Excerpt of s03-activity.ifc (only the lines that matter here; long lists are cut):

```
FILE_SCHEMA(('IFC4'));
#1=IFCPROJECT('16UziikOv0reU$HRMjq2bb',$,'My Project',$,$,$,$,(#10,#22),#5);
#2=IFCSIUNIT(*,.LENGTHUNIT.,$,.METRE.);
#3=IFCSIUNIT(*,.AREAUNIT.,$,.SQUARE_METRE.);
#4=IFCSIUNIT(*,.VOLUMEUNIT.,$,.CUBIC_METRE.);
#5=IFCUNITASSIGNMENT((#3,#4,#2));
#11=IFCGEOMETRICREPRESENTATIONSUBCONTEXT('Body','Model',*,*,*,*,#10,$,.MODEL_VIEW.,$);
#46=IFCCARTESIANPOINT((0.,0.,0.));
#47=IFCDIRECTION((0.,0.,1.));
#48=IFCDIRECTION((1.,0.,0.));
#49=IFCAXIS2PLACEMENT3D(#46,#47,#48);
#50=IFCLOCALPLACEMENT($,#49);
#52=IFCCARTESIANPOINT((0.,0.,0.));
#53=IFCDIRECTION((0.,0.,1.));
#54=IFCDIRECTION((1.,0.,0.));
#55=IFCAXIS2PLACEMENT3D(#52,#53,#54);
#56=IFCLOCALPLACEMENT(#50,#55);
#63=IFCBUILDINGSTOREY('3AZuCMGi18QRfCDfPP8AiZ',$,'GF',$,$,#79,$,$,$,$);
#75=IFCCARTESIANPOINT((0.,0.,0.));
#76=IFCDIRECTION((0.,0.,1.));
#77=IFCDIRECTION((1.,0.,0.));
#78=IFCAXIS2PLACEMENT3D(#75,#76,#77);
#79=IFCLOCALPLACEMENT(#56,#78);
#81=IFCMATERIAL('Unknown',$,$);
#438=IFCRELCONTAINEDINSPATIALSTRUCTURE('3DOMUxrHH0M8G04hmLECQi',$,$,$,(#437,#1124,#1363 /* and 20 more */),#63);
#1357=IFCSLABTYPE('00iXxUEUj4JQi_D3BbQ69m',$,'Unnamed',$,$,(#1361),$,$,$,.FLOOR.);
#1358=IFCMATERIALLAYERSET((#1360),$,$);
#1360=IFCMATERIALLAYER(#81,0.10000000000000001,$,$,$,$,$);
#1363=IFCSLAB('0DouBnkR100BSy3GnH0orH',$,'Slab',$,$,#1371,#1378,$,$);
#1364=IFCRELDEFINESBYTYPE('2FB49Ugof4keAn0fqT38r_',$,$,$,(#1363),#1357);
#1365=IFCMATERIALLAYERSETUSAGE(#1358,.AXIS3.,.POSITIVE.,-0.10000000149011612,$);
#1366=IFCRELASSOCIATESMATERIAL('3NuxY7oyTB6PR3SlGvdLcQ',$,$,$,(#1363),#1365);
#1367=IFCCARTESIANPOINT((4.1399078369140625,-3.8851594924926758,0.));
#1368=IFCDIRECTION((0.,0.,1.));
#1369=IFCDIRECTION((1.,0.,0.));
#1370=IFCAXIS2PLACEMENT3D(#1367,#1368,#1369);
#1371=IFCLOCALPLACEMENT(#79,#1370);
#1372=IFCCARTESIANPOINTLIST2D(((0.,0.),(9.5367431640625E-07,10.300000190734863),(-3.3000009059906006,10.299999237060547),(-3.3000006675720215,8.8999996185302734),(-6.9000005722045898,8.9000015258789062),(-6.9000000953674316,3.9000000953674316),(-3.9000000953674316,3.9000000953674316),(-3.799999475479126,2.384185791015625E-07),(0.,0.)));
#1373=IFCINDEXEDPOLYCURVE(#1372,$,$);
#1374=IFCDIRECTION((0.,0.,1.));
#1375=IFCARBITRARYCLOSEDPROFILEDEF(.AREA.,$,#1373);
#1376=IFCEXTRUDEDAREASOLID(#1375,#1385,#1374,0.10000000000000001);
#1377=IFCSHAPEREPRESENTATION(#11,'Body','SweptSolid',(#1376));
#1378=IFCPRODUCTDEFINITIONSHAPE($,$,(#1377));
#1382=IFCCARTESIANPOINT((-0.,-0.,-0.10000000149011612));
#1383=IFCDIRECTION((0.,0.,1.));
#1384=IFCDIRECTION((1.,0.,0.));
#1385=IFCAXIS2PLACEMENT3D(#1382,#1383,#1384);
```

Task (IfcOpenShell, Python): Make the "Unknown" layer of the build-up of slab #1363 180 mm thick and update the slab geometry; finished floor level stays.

```python
import ifcopenshell
import ifcopenshell.util.element
import ifcopenshell.util.representation
import ifcopenshell.util.unit

model = ifcopenshell.open("s03-activity.ifc")
unit_scale = ifcopenshell.util.unit.calculate_unit_scale(model)

layer_set = model.by_id(1358)
layer = next(l for l in layer_set.MaterialLayers if l.Material and l.Material.Name == "Unknown")
change = 0.18 / unit_scale - layer.LayerThickness
layer.LayerThickness += change

# Geometry does not follow the layer set by itself.
slabs = [e for e in ifcopenshell.util.element.get_elements_by_material(model, layer_set) if e.is_a("IfcSlab")]
for slab in sorted(slabs, key=lambda e: e.id()):
    body = ifcopenshell.util.representation.get_representation(slab, "Model", "Body")
    solid = body.Items[0]
    old_depth = solid.Depth
    solid.Depth += change
    # Extruded upwards: lower the start of the extrusion so the top stays.
    x, y, z = solid.Position.Location.Coordinates
    solid.Position.Location = model.createIfcCartesianPoint((x, y, z - change))
    print(slab.id(), f"{old_depth:g} -> {solid.Depth:g}")

# The layers are counted up from the underside, which has moved.
for usage in {ifcopenshell.util.element.get_material(slab) for slab in slabs}:
    usage.OffsetFromReferenceLine -= change

model.write("s03-activity-out.ifc")
```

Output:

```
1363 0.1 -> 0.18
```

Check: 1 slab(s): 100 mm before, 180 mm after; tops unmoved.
